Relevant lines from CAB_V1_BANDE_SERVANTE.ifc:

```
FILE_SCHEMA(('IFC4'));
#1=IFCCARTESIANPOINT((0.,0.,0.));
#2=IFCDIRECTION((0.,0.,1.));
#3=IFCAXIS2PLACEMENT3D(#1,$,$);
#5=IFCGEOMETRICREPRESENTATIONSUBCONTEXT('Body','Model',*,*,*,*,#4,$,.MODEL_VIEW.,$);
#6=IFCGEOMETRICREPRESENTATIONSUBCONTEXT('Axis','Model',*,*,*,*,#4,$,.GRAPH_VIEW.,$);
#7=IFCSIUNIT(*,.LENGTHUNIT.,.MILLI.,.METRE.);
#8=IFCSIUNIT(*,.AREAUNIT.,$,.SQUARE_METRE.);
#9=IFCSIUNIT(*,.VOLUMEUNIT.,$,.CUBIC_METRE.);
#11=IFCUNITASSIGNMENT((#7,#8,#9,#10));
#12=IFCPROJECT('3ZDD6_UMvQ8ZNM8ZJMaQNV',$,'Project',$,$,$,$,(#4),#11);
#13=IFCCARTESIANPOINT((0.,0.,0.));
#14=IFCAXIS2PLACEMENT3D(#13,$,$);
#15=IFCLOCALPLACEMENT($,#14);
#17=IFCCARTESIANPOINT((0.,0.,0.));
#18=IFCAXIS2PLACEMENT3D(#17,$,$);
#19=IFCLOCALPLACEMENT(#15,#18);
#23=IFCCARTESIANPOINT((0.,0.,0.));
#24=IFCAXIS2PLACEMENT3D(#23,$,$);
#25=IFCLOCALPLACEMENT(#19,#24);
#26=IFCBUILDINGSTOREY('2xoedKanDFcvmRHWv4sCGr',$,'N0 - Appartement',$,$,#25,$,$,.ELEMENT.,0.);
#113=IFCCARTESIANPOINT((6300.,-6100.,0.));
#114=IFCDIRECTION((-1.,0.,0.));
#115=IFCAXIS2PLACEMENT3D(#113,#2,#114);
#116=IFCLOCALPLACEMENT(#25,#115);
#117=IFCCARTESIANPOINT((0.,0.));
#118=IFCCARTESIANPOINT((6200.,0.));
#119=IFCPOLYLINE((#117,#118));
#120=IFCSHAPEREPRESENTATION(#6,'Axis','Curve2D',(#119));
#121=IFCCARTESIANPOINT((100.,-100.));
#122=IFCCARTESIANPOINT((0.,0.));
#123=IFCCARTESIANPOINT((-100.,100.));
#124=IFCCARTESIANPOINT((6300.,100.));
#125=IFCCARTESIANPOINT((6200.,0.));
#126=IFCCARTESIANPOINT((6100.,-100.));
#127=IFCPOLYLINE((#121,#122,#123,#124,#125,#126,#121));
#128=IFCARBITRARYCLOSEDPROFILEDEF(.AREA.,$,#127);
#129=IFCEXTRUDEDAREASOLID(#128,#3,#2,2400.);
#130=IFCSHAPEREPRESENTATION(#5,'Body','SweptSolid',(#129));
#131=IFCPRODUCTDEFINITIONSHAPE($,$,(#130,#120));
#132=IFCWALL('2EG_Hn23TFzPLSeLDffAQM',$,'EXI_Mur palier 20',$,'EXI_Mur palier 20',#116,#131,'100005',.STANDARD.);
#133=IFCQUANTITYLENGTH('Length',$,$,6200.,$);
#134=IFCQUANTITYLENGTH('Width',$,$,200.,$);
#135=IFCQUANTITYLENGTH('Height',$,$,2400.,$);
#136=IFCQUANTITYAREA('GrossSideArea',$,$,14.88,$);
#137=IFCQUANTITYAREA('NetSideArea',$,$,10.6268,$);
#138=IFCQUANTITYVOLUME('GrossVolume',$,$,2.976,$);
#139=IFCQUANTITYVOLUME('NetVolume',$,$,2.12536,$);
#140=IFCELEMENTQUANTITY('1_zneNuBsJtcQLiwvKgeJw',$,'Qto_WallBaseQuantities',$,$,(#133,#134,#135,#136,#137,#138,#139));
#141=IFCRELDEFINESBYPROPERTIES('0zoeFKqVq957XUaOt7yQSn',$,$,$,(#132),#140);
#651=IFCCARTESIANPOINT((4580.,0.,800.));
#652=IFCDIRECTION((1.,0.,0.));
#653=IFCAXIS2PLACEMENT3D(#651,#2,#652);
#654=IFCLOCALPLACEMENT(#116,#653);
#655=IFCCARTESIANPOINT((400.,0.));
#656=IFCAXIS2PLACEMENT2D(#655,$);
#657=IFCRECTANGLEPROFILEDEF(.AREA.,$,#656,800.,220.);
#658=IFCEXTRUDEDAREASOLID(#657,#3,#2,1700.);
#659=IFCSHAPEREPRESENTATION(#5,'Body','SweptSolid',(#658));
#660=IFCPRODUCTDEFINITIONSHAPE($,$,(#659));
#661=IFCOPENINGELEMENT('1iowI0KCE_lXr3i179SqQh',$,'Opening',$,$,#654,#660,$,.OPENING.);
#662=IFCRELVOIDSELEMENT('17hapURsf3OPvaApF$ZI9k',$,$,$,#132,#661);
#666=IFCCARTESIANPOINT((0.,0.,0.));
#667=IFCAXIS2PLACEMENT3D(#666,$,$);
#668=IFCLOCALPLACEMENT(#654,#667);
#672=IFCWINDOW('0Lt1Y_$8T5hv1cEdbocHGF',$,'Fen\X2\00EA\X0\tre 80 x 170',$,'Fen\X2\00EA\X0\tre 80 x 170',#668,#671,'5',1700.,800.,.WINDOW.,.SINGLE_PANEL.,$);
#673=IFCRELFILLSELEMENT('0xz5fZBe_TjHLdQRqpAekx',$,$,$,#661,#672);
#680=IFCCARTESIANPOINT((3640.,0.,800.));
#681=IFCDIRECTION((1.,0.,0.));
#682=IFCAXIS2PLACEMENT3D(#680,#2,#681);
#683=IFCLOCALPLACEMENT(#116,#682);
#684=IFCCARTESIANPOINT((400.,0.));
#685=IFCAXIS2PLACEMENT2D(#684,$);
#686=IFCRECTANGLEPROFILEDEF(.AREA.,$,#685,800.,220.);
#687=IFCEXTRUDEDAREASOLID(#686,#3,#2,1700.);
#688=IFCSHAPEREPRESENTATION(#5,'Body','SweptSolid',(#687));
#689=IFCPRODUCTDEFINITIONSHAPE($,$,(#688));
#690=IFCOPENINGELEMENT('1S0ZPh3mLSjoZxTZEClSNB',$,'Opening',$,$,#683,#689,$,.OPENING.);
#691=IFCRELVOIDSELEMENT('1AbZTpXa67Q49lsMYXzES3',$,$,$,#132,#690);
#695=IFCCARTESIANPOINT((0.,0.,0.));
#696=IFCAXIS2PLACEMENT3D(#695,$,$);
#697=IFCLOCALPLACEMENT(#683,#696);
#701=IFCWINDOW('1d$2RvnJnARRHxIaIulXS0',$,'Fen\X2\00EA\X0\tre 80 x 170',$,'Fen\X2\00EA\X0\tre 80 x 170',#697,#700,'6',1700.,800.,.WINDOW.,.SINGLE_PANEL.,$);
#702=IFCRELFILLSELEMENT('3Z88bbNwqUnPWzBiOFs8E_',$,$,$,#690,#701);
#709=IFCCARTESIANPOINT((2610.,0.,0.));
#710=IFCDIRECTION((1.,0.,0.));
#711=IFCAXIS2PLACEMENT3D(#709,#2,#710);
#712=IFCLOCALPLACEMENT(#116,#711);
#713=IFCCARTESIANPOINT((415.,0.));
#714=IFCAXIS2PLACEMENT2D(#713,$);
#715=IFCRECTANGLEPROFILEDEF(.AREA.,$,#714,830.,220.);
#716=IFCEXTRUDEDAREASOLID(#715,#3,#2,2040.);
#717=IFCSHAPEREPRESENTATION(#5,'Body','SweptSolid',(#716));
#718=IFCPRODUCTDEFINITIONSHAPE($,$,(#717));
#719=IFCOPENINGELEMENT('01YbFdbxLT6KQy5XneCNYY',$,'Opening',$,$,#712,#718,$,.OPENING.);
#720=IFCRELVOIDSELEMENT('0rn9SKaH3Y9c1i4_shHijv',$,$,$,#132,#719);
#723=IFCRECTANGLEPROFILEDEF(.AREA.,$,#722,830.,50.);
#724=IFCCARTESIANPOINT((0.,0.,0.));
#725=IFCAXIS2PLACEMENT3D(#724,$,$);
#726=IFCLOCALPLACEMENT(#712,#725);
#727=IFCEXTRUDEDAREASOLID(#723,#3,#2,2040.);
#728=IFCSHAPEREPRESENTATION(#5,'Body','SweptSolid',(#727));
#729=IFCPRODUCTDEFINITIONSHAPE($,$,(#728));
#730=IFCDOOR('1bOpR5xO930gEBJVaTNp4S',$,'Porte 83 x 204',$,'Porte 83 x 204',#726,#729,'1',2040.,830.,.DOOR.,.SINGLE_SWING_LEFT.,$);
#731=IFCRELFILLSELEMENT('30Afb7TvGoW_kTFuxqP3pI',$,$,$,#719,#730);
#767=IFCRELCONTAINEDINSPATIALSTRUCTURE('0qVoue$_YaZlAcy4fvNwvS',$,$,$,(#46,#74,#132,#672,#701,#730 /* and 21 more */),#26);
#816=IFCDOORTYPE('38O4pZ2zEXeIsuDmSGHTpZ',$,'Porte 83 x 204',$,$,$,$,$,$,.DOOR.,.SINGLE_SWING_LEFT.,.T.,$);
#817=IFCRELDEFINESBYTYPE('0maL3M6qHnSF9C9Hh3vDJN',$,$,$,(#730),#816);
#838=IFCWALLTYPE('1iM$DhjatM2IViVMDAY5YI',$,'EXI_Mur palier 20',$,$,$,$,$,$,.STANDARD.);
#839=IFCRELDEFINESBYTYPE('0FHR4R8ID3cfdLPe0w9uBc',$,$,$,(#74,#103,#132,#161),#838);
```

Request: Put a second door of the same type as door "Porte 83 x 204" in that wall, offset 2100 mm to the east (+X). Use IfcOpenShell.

```python
import ifcopenshell
import ifcopenshell.api.feature
import ifcopenshell.api.geometry
import ifcopenshell.api.pset
import ifcopenshell.api.root
import ifcopenshell.geom
import ifcopenshell.util.element
import ifcopenshell.util.placement
import ifcopenshell.util.shape
import ifcopenshell.util.unit

model = ifcopenshell.open("CAB_V1_BANDE_SERVANTE.ifc")
unit_scale = ifcopenshell.util.unit.calculate_unit_scale(model)
area_scale = ifcopenshell.util.unit.calculate_unit_scale(model, "AREAUNIT")
volume_scale = ifcopenshell.util.unit.calculate_unit_scale(model, "VOLUMEUNIT")
settings = ifcopenshell.geom.settings()


def volume(element):
    """Net volume in cubic metres, openings subtracted."""
    shape = ifcopenshell.geom.create_shape(settings, element)
    return ifcopenshell.util.shape.get_volume(shape.geometry)


door = model.by_id(730)
opening = door.FillsVoids[0].RelatingOpeningElement
wall = opening.VoidsElements[0].RelatingBuildingElement
before = volume(wall)
shift = ifcopenshell.util.placement.get_local_placement(wall.ObjectPlacement)[:3, 0] * -2.1 / unit_scale

# copy_class copies the void relationship, type, container and properties, but no geometry.
new_opening = ifcopenshell.api.root.copy_class(model, product=opening)
new_opening.Representation = ifcopenshell.util.element.copy_deep(
    model, opening.Representation, exclude=["IfcGeometricRepresentationContext", "IfcRepresentationMap"]
)
new_door = ifcopenshell.api.root.copy_class(model, product=door)
new_door.Representation = ifcopenshell.util.element.copy_deep(
    model, door.Representation, exclude=["IfcGeometricRepresentationContext", "IfcRepresentationMap"]
)
new_door.Tag = None
ifcopenshell.api.feature.add_filling(model, opening=new_opening, element=new_door)

for old, new in ((opening, new_opening), (door, new_door)):
    matrix = ifcopenshell.util.placement.get_local_placement(old.ObjectPlacement)
    matrix[:3, 3] += shift
    ifcopenshell.api.geometry.edit_object_placement(model, product=new, matrix=matrix, is_si=False)

after = volume(wall)
thickness = 0.2  # wall thickness in metres

# Update the wall's stored quantities.
qto = model.by_id(ifcopenshell.util.element.get_pset(wall, "Qto_WallBaseQuantities", should_inherit=False)["id"])
ifcopenshell.api.pset.edit_qto(model, qto=qto, properties={
    "NetSideArea": after / thickness / area_scale,
    "NetVolume": after / volume_scale,
})

print(f"wall volume {before:.3f} -> {after:.3f} m3")

model.write("CAB_V1_BANDE_SERVANTE_updated.ifc")
```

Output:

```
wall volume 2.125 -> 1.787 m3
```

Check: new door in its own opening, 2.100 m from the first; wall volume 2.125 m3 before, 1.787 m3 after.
